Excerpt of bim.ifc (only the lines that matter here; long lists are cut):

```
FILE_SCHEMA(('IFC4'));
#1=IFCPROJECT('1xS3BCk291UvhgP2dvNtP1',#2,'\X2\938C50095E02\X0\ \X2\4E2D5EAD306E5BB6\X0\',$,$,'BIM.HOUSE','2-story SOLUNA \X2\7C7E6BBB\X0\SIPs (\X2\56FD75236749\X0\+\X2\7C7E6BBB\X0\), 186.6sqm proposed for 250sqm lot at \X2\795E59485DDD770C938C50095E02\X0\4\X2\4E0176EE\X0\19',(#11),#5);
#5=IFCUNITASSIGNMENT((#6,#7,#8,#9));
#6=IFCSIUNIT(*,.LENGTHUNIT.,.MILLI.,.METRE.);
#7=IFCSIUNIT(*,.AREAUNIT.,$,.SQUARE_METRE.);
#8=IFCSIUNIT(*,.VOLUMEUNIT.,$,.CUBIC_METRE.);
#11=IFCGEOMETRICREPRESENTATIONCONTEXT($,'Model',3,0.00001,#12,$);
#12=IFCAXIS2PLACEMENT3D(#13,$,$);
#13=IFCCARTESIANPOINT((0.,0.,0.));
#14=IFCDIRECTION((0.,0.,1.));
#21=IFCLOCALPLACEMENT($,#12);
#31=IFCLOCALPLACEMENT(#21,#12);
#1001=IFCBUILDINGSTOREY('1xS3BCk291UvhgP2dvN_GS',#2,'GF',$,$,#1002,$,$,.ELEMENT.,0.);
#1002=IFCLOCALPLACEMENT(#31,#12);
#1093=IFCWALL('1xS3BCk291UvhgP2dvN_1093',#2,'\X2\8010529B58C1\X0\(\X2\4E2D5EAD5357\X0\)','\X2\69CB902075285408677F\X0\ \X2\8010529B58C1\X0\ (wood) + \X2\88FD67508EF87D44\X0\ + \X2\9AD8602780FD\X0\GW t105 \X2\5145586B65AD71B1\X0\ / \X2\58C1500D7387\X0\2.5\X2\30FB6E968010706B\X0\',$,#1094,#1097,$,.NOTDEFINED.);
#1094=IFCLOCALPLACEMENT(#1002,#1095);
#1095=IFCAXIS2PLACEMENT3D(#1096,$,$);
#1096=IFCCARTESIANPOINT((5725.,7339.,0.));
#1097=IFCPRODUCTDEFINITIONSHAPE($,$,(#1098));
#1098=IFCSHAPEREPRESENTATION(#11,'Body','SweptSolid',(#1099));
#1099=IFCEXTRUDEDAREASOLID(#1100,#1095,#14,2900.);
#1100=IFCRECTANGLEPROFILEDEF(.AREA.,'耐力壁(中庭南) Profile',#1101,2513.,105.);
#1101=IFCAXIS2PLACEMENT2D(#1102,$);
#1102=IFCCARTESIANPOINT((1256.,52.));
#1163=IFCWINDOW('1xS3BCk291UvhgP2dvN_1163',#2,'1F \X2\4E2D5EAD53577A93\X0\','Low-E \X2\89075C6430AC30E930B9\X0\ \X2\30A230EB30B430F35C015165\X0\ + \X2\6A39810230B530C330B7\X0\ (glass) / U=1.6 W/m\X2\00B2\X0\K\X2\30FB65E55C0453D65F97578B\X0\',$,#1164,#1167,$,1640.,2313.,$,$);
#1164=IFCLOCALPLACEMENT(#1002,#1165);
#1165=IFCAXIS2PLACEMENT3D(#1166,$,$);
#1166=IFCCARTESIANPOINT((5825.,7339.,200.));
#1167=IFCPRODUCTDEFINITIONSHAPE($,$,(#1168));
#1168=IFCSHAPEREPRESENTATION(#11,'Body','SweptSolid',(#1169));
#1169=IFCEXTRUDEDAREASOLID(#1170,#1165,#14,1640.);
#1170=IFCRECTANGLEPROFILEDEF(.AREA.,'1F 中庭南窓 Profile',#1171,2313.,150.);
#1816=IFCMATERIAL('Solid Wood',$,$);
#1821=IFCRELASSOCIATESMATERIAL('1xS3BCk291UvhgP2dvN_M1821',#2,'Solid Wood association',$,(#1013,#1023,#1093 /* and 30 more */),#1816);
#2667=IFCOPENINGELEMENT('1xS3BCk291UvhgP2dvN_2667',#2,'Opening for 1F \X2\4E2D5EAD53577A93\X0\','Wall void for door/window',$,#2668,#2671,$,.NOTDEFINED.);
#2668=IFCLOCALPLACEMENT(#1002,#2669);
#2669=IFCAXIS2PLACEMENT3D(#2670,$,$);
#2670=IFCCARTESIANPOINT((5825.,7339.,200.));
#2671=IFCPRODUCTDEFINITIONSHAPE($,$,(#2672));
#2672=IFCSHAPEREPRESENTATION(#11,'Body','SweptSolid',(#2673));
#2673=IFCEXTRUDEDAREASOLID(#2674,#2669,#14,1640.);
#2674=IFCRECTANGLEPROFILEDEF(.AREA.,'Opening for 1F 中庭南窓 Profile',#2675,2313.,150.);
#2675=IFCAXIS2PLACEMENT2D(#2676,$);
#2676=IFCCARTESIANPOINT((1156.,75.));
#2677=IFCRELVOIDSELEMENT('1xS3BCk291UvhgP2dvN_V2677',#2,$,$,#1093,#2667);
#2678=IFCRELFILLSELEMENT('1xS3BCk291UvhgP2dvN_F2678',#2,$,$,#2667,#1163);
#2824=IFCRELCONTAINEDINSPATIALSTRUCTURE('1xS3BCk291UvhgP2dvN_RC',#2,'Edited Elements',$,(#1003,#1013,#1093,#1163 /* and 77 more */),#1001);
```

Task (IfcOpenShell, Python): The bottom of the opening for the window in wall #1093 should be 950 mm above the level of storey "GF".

```python
import numpy as np
import ifcopenshell
import ifcopenshell.api.geometry
import ifcopenshell.geom
import ifcopenshell.util.element
import ifcopenshell.util.placement
import ifcopenshell.util.shape
import ifcopenshell.util.unit

model = ifcopenshell.open("bim.ifc")
unit_scale = ifcopenshell.util.unit.calculate_unit_scale(model)

window = model.by_id(1163)
opening = window.FillsVoids[0].RelatingOpeningElement
storey = ifcopenshell.util.element.get_container(window, ifc_class="IfcBuildingStorey")
level = ifcopenshell.util.placement.get_local_placement(storey.ObjectPlacement)[2, 3]

# The opening's origin need not be at the sill, so measure its lowest point.
shape = ifcopenshell.geom.create_shape(ifcopenshell.geom.settings(), opening)
bottom = ifcopenshell.util.shape.get_shape_bottom_elevation(shape, shape.geometry) / unit_scale
dz = level + 0.95 / unit_scale - bottom

shift = np.array([0.0, 0.0, dz])
# The window is not placed relative to its opening, so move both.
for product in (opening, window):
    matrix = ifcopenshell.util.placement.get_local_placement(product.ObjectPlacement)
    matrix[:3, 3] += shift
    ifcopenshell.api.geometry.edit_object_placement(model, product=product, matrix=matrix, is_si=False)

print(f"moved by {dz * unit_scale:+.3f} m")

model.write("bim_edited.ifc")
```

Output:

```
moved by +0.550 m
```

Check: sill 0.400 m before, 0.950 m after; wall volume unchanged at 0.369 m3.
